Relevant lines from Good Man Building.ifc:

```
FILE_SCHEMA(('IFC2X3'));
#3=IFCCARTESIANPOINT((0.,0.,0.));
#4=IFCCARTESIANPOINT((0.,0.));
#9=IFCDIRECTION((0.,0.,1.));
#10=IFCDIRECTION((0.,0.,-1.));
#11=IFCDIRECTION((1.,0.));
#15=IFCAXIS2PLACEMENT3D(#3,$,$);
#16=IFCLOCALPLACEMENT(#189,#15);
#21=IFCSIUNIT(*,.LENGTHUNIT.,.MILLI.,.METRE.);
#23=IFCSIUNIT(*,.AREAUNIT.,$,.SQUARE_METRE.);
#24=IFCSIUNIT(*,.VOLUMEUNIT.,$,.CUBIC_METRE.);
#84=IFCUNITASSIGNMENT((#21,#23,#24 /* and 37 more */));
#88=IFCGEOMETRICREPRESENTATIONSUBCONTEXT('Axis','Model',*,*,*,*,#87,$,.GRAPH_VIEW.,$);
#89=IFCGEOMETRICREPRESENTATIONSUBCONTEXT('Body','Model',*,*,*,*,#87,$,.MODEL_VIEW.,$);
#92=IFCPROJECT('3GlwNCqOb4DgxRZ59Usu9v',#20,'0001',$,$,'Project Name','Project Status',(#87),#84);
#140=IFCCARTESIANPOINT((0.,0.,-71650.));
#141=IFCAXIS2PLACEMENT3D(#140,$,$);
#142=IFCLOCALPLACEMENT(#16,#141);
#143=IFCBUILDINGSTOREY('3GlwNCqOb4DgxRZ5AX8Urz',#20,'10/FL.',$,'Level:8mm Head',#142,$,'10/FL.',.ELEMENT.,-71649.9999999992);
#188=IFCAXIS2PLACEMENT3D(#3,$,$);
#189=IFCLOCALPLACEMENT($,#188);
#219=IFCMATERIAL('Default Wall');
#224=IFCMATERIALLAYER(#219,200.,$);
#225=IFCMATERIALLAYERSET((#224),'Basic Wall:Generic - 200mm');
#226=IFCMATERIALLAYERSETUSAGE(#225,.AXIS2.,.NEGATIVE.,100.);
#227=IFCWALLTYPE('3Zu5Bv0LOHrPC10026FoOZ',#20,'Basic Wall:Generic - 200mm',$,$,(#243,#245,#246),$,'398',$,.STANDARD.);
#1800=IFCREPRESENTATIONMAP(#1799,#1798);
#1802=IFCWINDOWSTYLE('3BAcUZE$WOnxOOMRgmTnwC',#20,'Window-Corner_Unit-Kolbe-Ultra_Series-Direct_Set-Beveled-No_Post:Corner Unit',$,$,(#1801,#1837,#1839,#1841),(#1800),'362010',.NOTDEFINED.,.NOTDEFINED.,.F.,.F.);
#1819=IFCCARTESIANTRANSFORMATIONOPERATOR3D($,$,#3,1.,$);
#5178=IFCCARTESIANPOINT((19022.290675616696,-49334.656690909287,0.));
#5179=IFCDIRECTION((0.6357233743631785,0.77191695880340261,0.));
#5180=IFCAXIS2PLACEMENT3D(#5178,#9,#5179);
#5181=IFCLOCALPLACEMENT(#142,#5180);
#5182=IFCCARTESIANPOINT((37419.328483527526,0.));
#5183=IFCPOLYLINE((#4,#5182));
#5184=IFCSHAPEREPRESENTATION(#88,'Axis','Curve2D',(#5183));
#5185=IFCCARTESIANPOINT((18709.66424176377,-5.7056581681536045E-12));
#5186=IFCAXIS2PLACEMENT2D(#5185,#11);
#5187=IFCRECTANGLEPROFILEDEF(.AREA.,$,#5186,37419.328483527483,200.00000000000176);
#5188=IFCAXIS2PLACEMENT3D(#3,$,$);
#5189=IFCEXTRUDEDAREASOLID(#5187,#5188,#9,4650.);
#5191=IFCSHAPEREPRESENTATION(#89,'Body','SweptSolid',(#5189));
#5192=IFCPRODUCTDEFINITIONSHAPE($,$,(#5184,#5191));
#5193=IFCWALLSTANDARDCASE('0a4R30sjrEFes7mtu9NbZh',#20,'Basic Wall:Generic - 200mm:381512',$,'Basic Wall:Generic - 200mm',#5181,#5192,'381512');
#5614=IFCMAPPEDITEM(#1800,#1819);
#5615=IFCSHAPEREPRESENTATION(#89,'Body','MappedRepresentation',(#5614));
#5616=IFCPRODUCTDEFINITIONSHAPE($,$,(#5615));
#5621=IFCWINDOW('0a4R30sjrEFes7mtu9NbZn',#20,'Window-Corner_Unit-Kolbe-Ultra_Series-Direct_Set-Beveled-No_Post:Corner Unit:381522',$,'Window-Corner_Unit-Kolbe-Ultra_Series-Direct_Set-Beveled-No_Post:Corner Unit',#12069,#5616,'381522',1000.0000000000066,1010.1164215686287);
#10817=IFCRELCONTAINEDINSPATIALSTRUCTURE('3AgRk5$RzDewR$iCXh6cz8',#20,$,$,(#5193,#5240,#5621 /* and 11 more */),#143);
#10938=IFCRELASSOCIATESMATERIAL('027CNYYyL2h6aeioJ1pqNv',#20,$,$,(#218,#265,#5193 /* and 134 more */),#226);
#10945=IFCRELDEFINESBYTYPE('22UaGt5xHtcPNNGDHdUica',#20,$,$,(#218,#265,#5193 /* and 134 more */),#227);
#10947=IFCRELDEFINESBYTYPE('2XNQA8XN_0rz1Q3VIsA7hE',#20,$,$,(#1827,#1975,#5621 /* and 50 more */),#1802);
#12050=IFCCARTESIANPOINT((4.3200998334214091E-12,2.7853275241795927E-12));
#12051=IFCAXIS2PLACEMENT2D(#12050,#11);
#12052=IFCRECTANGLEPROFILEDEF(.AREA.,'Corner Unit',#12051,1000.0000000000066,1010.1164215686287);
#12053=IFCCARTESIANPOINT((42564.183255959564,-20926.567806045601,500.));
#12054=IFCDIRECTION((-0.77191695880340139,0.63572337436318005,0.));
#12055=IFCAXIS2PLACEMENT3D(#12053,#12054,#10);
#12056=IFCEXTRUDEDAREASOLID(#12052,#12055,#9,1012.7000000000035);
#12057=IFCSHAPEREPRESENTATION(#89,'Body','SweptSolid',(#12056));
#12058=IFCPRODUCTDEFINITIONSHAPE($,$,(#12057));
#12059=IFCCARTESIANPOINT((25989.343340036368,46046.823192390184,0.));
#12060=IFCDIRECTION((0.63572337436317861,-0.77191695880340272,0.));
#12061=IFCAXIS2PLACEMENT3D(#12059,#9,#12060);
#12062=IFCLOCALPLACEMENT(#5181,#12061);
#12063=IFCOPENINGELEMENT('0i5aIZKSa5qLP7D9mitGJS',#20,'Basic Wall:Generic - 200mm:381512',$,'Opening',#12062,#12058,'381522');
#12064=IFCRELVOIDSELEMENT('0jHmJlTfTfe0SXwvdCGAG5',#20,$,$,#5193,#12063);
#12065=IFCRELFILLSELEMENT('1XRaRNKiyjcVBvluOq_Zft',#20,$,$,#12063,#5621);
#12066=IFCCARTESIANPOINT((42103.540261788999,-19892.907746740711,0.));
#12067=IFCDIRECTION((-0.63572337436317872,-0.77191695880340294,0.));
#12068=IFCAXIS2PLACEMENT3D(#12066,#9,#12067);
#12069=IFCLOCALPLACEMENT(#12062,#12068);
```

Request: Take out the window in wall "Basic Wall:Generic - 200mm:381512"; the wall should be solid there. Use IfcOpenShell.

```python
import ifcopenshell
import ifcopenshell.api.feature
import ifcopenshell.api.root
import ifcopenshell.geom
import ifcopenshell.util.shape

model = ifcopenshell.open("Good Man Building.ifc")
settings = ifcopenshell.geom.settings()


def volume(element):
    """Net volume in cubic metres, openings subtracted."""
    shape = ifcopenshell.geom.create_shape(settings, element)
    return ifcopenshell.util.shape.get_volume(shape.geometry)


window = model.by_id(5621)
opening = window.FillsVoids[0].RelatingOpeningElement
wall = opening.VoidsElements[0].RelatingBuildingElement
before = volume(wall)

ifcopenshell.api.root.remove_product(model, product=window)
ifcopenshell.api.feature.remove_feature(model, feature=opening)

after = volume(wall)

print(f"wall volume {before:.3f} -> {after:.3f} m3")

model.write("Good Man Building_rev.ifc")
```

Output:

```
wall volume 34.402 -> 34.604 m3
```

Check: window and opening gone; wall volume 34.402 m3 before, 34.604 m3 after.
